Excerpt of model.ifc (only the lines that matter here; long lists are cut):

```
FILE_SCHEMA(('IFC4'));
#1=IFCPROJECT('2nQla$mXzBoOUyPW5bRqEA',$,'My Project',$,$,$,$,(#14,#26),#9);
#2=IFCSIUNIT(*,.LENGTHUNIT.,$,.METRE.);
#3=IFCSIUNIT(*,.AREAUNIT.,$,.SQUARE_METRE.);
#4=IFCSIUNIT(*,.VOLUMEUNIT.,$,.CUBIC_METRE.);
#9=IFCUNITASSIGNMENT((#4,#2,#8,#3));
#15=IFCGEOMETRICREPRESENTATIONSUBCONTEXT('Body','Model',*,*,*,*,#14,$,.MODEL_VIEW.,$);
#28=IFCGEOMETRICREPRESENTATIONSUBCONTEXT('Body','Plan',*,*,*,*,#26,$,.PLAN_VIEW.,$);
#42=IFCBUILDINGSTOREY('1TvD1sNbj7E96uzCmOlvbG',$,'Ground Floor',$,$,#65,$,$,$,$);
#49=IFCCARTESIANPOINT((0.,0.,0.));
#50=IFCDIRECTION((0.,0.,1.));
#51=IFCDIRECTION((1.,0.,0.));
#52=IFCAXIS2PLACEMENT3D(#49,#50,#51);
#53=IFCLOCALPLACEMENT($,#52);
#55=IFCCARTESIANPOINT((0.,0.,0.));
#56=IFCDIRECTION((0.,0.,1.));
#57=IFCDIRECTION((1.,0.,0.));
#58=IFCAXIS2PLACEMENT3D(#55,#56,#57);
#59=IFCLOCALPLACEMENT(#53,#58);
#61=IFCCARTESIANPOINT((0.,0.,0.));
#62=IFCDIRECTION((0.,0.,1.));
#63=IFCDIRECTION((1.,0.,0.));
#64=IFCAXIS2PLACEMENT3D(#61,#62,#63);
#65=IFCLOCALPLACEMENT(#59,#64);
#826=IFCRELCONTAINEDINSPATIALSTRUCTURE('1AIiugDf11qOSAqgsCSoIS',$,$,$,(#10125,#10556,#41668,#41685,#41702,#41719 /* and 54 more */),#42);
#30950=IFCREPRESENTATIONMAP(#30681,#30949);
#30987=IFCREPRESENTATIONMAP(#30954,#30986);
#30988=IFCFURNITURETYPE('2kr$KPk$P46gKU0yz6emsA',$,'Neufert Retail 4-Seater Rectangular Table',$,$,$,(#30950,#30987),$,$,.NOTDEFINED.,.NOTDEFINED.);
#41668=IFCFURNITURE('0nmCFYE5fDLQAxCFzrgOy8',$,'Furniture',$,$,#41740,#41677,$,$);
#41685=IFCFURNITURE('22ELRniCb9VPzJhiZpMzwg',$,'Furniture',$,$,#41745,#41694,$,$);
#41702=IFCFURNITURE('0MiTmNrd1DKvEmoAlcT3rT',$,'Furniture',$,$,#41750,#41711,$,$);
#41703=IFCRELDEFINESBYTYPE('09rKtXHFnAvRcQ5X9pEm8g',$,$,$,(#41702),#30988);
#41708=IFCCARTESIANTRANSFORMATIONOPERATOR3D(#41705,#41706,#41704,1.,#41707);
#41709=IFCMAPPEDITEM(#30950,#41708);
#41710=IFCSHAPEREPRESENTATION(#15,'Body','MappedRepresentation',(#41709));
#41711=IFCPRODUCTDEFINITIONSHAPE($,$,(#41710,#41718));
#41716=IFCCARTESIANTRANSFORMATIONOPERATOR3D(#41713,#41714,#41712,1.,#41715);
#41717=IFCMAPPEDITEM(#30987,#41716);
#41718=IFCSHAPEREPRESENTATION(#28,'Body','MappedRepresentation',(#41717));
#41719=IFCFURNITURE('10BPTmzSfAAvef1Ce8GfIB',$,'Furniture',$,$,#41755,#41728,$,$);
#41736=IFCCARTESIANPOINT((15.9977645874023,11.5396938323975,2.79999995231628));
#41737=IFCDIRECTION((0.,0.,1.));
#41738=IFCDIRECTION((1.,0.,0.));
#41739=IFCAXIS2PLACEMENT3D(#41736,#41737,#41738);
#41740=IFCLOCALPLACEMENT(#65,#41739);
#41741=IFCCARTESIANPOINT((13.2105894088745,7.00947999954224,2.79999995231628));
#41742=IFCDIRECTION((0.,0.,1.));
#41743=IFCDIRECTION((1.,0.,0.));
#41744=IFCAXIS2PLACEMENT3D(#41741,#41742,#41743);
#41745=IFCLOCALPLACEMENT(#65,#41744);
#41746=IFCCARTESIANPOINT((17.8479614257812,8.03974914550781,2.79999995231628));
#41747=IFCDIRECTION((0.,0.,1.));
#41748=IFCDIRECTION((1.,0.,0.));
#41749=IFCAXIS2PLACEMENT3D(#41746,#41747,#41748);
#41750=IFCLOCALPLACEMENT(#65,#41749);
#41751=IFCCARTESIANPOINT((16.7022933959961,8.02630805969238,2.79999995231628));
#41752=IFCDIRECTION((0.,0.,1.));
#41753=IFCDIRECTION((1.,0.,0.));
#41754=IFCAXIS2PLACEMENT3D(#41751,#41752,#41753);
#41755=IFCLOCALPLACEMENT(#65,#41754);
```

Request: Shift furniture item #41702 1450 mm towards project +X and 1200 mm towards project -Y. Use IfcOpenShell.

```python
import ifcopenshell
import ifcopenshell.api.geometry
import ifcopenshell.util.placement

model = ifcopenshell.open("model.ifc")

item = model.by_guid("0MiTmNrd1DKvEmoAlcT3rT")
matrix = ifcopenshell.util.placement.get_local_placement(item.ObjectPlacement)
matrix[0, 3] += 1.45
matrix[1, 3] -= 1.2
ifcopenshell.api.geometry.edit_object_placement(model, product=item, matrix=matrix, is_si=False)

print(ifcopenshell.util.placement.get_local_placement(item.ObjectPlacement).round(3) + 0.0)

model.write("model_v2.ifc")
```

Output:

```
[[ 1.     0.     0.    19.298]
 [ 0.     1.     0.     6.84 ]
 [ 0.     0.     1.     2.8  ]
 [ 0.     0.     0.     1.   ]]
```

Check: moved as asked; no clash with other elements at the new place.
